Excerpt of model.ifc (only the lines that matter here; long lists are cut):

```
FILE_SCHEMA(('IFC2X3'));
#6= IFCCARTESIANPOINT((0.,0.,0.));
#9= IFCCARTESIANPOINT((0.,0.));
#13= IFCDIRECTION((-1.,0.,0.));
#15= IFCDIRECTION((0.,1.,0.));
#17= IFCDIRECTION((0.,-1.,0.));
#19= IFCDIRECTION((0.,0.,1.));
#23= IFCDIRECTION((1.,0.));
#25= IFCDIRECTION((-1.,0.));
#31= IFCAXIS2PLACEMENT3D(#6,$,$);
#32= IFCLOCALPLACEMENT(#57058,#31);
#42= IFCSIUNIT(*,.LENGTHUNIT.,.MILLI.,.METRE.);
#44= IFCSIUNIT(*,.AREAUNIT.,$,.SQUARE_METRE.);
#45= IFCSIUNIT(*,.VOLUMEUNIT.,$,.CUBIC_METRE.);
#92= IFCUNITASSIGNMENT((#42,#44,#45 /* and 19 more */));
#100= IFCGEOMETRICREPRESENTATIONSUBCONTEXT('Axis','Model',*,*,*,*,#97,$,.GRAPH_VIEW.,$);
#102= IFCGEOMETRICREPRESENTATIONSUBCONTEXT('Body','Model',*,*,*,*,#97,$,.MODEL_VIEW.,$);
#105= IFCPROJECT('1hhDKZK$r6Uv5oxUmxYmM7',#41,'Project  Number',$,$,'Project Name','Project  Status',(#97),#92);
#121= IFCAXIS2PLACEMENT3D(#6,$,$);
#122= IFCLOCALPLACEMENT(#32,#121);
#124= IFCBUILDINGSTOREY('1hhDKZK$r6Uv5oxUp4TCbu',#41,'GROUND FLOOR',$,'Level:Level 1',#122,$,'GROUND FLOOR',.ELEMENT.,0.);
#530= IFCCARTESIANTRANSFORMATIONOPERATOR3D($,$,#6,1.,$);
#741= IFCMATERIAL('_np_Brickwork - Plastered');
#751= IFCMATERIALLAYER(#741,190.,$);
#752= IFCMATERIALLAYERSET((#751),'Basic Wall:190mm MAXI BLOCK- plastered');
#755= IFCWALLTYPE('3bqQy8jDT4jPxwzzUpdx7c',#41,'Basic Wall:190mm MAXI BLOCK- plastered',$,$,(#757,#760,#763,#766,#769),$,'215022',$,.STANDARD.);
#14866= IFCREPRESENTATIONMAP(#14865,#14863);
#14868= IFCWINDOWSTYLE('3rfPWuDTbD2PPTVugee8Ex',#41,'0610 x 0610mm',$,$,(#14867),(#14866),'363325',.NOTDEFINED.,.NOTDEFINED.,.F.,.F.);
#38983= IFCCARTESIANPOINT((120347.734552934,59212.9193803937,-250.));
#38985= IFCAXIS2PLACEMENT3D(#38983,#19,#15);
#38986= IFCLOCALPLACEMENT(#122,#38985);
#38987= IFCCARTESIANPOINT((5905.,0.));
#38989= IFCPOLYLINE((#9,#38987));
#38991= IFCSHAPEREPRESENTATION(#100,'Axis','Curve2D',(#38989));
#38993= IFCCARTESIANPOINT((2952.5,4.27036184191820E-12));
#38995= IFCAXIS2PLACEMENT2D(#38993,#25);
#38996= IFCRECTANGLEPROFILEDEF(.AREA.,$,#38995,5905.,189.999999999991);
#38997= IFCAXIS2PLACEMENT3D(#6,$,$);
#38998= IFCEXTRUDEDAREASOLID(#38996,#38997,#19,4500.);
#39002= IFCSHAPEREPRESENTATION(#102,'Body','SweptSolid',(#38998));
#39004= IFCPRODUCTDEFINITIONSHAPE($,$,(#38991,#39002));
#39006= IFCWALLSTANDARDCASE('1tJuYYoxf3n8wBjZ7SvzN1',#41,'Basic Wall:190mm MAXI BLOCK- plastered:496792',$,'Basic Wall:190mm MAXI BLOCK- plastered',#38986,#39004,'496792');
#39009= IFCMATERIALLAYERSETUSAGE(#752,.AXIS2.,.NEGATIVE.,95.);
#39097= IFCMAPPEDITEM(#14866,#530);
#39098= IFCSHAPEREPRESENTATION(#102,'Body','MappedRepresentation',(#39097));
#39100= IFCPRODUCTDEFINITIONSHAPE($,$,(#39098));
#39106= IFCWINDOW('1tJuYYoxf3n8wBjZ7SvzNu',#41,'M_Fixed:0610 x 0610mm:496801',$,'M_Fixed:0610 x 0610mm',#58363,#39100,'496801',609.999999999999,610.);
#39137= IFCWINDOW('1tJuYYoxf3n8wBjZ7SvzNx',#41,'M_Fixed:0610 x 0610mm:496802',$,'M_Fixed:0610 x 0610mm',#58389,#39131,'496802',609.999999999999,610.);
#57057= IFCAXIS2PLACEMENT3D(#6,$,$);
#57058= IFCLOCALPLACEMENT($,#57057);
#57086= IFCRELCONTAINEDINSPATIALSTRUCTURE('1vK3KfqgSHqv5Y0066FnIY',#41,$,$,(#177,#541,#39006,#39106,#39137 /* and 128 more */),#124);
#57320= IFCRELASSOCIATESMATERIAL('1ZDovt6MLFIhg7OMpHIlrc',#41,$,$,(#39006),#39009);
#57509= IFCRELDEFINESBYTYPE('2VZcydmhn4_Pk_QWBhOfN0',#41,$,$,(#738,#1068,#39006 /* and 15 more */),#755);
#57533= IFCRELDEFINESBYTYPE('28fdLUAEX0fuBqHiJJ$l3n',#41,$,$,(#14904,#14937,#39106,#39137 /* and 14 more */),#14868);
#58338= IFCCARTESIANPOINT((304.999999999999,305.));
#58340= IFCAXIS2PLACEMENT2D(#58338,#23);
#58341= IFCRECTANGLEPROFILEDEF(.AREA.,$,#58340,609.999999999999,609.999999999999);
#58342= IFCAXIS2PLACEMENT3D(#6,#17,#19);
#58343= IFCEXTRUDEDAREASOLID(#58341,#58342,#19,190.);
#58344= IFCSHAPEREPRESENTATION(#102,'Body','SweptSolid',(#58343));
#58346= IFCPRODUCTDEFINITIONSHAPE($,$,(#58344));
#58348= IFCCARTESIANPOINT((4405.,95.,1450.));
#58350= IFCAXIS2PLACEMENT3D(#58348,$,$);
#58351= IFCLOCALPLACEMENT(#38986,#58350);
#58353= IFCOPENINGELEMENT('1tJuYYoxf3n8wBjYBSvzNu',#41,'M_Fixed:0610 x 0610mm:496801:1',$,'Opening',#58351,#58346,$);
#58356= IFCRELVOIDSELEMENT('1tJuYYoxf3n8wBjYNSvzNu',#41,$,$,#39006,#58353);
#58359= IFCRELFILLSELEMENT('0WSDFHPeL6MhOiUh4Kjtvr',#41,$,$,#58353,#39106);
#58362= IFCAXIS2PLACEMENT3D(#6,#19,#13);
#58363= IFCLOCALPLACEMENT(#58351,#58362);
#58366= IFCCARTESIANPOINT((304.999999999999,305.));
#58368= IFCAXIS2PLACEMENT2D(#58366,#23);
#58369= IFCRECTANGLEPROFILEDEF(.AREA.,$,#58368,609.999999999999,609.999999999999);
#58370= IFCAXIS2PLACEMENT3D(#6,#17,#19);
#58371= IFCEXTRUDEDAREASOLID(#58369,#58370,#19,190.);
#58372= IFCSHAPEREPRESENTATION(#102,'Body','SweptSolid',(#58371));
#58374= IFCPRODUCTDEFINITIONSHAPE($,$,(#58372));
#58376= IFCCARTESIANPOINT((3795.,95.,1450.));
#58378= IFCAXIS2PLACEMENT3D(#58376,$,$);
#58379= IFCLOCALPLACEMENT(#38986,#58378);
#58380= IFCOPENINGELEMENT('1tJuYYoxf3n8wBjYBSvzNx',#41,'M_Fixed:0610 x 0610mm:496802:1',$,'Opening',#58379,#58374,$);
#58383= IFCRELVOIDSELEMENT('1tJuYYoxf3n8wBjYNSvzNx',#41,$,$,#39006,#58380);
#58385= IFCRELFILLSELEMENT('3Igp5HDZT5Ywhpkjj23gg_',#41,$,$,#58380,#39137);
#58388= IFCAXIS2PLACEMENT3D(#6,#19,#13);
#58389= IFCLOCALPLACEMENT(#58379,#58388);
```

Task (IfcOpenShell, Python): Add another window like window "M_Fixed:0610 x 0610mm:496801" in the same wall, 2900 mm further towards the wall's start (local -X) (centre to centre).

```python
import ifcopenshell
import ifcopenshell.api.feature
import ifcopenshell.api.geometry
import ifcopenshell.api.root
import ifcopenshell.geom
import ifcopenshell.util.element
import ifcopenshell.util.placement
import ifcopenshell.util.shape

model = ifcopenshell.open("model.ifc")
settings = ifcopenshell.geom.settings()


def volume(element):
    """Net volume in cubic metres, openings subtracted."""
    shape = ifcopenshell.geom.create_shape(settings, element)
    return ifcopenshell.util.shape.get_volume(shape.geometry)


def reuse_history(source, copy):
    """copy_class also copies each property set's owner history, people and application; keep the originals."""
    for rel in copy.IsDefinedBy:
        if rel.is_a("IfcRelDefinesByProperties") and (history := rel.RelatingPropertyDefinition.OwnerHistory):
            rel.RelatingPropertyDefinition.OwnerHistory = source.OwnerHistory
            ifcopenshell.util.element.remove_deep2(model, history)


window = model.by_id(39106)
opening = window.FillsVoids[0].RelatingOpeningElement
wall = opening.VoidsElements[0].RelatingBuildingElement
before = volume(wall)
shift = ifcopenshell.util.placement.get_local_placement(wall.ObjectPlacement)[:3, 0] * -2900.0

# copy_class copies the void relationship, type, container and properties, but no geometry.
new_opening = ifcopenshell.api.root.copy_class(model, product=opening)
new_opening.Representation = ifcopenshell.util.element.copy_deep(
    model, opening.Representation, exclude=["IfcGeometricRepresentationContext", "IfcRepresentationMap"]
)
new_opening.Name = "M_Fixed:0610 x 0610mm"
new_window = ifcopenshell.api.root.copy_class(model, product=window)
new_window.Representation = ifcopenshell.util.element.copy_deep(
    model, window.Representation, exclude=["IfcGeometricRepresentationContext", "IfcRepresentationMap"]
)
new_window.Name = "M_Fixed:0610 x 0610mm"
new_window.Tag = None
reuse_history(window, new_window)
fills = ifcopenshell.api.feature.add_filling(model, opening=new_opening, element=new_window)
fills.OwnerHistory = new_window.OwnerHistory  # required in IFC2X3

for old, new in ((opening, new_opening), (window, new_window)):
    matrix = ifcopenshell.util.placement.get_local_placement(old.ObjectPlacement)
    matrix[:3, 3] += shift
    ifcopenshell.api.geometry.edit_object_placement(model, product=new, matrix=matrix, is_si=False)

after = volume(wall)

print(f"wall volume {before:.3f} -> {after:.3f} m3")

model.write("model_v2.ifc")
```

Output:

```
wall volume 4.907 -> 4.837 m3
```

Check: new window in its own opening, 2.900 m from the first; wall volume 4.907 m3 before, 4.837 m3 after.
